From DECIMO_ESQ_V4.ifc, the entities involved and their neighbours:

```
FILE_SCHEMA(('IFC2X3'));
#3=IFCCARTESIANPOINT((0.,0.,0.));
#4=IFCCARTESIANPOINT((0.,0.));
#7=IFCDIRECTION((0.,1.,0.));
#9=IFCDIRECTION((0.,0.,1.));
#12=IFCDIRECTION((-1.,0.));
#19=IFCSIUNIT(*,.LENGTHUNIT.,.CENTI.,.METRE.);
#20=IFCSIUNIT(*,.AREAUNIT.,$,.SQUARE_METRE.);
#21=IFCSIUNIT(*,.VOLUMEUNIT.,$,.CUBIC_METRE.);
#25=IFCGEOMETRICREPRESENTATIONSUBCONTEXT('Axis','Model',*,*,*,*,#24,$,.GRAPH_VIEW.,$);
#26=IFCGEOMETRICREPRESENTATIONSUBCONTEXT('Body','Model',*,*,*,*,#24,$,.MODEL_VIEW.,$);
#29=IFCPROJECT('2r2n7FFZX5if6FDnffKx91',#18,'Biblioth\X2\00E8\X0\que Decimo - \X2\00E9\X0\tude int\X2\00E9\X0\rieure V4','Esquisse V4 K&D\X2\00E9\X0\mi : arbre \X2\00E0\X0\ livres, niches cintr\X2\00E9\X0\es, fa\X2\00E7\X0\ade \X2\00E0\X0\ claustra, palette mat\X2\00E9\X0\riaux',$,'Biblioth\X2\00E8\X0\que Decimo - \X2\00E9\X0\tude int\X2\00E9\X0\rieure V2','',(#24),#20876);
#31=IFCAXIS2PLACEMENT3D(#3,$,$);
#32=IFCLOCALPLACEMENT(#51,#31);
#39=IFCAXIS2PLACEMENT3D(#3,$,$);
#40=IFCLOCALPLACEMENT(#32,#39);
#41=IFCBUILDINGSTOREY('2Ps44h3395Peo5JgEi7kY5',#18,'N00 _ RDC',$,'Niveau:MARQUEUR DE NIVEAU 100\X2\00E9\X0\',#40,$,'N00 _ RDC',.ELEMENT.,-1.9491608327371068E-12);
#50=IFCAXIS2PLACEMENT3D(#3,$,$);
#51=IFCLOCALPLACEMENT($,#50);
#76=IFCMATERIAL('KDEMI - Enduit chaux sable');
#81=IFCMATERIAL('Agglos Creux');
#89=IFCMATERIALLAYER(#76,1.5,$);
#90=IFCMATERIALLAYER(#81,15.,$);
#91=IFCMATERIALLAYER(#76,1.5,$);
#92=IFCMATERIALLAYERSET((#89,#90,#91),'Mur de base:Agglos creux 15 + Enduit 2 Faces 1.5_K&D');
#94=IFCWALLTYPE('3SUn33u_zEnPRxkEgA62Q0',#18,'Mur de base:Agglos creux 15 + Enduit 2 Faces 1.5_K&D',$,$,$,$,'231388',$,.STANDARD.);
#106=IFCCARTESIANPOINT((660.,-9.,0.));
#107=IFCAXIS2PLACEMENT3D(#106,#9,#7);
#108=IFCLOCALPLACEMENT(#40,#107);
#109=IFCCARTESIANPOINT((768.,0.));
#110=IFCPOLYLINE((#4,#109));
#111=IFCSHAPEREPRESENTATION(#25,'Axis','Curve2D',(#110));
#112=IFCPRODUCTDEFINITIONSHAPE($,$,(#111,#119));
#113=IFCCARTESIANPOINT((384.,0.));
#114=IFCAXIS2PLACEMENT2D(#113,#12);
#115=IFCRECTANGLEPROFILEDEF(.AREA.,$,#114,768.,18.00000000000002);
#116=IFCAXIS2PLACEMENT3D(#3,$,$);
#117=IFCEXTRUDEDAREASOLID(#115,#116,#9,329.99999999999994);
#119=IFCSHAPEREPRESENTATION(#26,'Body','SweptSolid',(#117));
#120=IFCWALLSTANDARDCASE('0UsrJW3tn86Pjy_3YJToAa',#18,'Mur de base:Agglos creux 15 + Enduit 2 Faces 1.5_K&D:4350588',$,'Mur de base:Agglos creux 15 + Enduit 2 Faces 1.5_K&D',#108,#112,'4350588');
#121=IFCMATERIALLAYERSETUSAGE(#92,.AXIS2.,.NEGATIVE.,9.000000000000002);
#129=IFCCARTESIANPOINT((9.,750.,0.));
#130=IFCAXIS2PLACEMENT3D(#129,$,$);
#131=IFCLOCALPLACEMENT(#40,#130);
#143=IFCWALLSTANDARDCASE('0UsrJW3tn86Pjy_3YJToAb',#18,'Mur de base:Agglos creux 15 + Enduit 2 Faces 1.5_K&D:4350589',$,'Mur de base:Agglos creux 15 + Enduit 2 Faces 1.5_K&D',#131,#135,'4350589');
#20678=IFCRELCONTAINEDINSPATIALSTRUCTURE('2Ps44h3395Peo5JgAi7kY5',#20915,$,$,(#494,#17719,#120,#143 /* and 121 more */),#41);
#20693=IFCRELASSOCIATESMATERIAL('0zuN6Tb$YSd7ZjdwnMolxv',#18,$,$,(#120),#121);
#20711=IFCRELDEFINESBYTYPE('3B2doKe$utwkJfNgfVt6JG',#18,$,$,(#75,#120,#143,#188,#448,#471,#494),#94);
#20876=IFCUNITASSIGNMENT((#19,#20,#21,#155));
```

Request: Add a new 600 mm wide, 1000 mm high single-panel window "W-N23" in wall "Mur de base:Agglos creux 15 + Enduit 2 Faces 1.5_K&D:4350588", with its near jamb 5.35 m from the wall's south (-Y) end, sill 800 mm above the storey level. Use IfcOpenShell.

```python
import numpy as np
import ifcopenshell
import ifcopenshell.api.feature
import ifcopenshell.api.geometry
import ifcopenshell.api.root
import ifcopenshell.api.spatial
import ifcopenshell.api.type
import ifcopenshell.geom
import ifcopenshell.util.element
import ifcopenshell.util.placement
import ifcopenshell.util.representation
import ifcopenshell.util.shape
import ifcopenshell.util.unit

model = ifcopenshell.open("DECIMO_ESQ_V4.ifc")
unit_scale = ifcopenshell.util.unit.calculate_unit_scale(model)
settings = ifcopenshell.geom.settings()


def volume(element):
    """Net volume in cubic metres, openings subtracted."""
    shape = ifcopenshell.geom.create_shape(settings, element)
    return ifcopenshell.util.shape.get_volume(shape.geometry)


wall = model.by_guid("0UsrJW3tn86Pjy_3YJToAa")
storey = ifcopenshell.util.element.get_container(wall, ifc_class="IfcBuildingStorey")
context = ifcopenshell.util.representation.get_context(model, "Model", "Body", "MODEL_VIEW")
before = volume(wall)

width, height, from_end, sill = 0.6, 1, 5.35, 0.8  # metres

# The wall runs along its own X axis, and the end named is its -X end.
wall_shape = ifcopenshell.geom.create_shape(settings, wall)
x, y, z = ifcopenshell.util.shape.get_vertices(wall_shape.geometry).T
start = x.min() + from_end
face, thickness = float(y.min()), float(y.max() - y.min())
wall_matrix = ifcopenshell.util.placement.get_local_placement(wall.ObjectPlacement)
level = ifcopenshell.util.placement.get_local_placement(storey.ObjectPlacement)[2, 3]


def in_wall(x, y):
    """Placement at x, y metres in the wall's axes, at sill height."""
    matrix = wall_matrix.copy()
    matrix[:, 3] = wall_matrix @ np.array([x / unit_scale, y / unit_scale, 0.0, 1.0])
    matrix[2, 3] = level + sill / unit_scale
    return matrix


# Opening: a box that overshoots both wall faces by 50 mm.
opening = ifcopenshell.api.root.create_entity(model, ifc_class="IfcOpeningElement")
box = ifcopenshell.api.geometry.add_wall_representation(
    model, context=context, length=width, height=height, thickness=thickness + 0.1
)
ifcopenshell.api.geometry.assign_representation(model, product=opening, representation=box)
ifcopenshell.api.geometry.edit_object_placement(model, product=opening, matrix=in_wall(start, face - 0.05), is_si=False)
ifcopenshell.api.feature.add_feature(model, feature=opening, element=wall)

window = ifcopenshell.api.root.create_entity(model, ifc_class="IfcWindow", name="W-N23")
window.OverallWidth, window.OverallHeight = width / unit_scale, height / unit_scale
body = ifcopenshell.api.geometry.add_window_representation(
    model,
    context=context,
    overall_width=window.OverallWidth,
    overall_height=window.OverallHeight,
    partition_type="SINGLE_PANEL",
)
ifcopenshell.api.geometry.assign_representation(model, product=window, representation=body)
ifcopenshell.api.spatial.assign_container(model, products=[window], relating_structure=storey)
fills = ifcopenshell.api.feature.add_filling(model, opening=opening, element=window)
fills.OwnerHistory = window.OwnerHistory  # required in IFC2X3

# IFC2X3 keeps the operation on the window style.
style = ifcopenshell.api.root.create_entity(model, ifc_class="IfcWindowStyle", name="W-N23")
style.OperationType, style.ConstructionType = "SINGLE_PANEL", "NOTDEFINED"
style.ParameterTakesPrecedence = style.Sizeable = False
ifcopenshell.api.type.assign_type(model, related_objects=[window], relating_type=style)

# Centre the window in the wall's thickness.
ifcopenshell.api.geometry.edit_object_placement(model, product=window, matrix=in_wall(start, face), is_si=False)
window_shape = ifcopenshell.geom.create_shape(settings, window)
depth = ifcopenshell.util.shape.get_vertices(window_shape.geometry)[:, 1]
offset = face + thickness / 2 - (depth.min() + depth.max()) / 2
ifcopenshell.api.geometry.edit_object_placement(model, product=window, matrix=in_wall(start, offset), is_si=False)

after = volume(wall)

print(f"wall volume {before:.3f} -> {after:.3f} m3")

model.write("DECIMO_ESQ_V4_edited.ifc")
```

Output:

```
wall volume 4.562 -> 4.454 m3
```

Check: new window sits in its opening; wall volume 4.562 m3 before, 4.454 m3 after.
